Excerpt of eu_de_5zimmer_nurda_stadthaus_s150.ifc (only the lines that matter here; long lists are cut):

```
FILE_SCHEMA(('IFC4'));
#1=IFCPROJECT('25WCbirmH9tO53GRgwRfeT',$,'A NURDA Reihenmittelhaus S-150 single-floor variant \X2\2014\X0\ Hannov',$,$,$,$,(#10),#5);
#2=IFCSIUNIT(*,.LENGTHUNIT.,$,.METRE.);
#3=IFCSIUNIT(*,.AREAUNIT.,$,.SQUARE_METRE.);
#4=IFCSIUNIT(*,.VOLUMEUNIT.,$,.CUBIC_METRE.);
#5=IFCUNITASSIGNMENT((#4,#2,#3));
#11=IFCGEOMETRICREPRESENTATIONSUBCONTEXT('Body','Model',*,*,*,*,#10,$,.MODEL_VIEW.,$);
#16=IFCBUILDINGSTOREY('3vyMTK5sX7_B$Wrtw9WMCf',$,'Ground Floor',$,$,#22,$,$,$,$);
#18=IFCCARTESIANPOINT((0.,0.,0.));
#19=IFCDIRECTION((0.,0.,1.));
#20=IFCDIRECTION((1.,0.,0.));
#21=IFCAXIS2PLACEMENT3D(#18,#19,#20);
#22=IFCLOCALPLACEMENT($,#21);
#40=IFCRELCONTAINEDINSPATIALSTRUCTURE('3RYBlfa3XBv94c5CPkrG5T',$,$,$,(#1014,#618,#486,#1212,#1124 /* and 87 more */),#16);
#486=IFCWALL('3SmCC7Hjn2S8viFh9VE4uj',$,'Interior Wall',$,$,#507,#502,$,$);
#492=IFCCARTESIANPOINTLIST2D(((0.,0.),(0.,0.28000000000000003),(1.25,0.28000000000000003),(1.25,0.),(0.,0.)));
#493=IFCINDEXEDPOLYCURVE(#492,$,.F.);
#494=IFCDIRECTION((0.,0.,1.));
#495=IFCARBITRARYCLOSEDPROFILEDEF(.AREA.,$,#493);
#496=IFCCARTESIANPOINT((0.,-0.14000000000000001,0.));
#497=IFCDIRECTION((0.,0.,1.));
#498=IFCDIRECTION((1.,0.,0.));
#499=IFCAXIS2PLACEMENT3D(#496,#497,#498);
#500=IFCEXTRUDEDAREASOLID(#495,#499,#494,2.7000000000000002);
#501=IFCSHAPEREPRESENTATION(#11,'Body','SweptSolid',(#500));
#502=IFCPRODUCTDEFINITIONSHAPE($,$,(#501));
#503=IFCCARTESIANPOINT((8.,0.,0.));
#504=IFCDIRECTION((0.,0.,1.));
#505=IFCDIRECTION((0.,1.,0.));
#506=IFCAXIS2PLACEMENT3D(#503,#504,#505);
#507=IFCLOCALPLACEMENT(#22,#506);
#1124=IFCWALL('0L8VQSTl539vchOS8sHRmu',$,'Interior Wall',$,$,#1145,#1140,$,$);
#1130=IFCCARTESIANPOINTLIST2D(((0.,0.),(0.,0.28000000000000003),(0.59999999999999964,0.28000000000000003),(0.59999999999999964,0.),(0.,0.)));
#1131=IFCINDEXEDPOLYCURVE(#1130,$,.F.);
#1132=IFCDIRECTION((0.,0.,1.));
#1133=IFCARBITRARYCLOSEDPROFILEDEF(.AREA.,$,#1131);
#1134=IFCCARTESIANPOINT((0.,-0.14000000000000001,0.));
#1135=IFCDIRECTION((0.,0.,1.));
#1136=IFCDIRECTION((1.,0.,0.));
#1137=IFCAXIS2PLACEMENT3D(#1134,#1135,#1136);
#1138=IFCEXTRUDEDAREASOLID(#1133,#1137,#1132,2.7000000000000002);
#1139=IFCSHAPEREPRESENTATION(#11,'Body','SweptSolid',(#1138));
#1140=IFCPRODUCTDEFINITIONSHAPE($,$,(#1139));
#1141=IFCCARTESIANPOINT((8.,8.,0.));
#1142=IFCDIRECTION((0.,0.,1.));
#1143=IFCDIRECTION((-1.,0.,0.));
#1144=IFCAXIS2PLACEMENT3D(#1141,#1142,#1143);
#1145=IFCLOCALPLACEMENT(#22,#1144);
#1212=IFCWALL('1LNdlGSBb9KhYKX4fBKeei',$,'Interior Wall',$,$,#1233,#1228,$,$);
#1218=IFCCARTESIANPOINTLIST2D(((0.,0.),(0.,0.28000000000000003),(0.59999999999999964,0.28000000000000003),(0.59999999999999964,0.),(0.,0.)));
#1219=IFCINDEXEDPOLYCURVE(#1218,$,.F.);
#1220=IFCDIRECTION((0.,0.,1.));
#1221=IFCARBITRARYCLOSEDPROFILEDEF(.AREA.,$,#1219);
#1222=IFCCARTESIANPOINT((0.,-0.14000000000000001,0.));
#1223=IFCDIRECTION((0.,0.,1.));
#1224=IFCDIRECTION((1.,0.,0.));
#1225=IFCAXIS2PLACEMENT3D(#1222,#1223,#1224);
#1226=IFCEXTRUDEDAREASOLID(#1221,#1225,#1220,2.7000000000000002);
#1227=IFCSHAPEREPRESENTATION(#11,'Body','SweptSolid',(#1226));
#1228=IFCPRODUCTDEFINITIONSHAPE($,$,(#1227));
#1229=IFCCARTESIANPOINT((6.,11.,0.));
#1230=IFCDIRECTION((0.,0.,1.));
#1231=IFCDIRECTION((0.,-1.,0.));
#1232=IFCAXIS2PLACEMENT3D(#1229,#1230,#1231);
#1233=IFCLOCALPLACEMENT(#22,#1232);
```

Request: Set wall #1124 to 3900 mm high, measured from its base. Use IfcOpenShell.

```python
import ifcopenshell
import ifcopenshell.geom
import ifcopenshell.util.representation
import ifcopenshell.util.shape

model = ifcopenshell.open("eu_de_5zimmer_nurda_stadthaus_s150.ifc")
settings = ifcopenshell.geom.settings()


def volume(element):
    """Net volume in cubic metres, openings subtracted."""
    shape = ifcopenshell.geom.create_shape(settings, element)
    return ifcopenshell.util.shape.get_volume(shape.geometry)


wall = model.by_guid("0L8VQSTl539vchOS8sHRmu")
before = volume(wall)

body = ifcopenshell.util.representation.get_representation(wall, "Model", "Body")
solid = body.Items[0]
old_height = solid.Depth
solid.Depth = 3.9
after = volume(wall)

print(f"height {old_height:g} -> {solid.Depth:g}, volume {before:.3f} -> {after:.3f} m3")

model.write("eu_de_5zimmer_nurda_stadthaus_s150_updated.ifc")
```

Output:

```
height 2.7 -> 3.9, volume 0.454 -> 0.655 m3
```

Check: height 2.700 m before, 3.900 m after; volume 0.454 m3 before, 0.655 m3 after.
